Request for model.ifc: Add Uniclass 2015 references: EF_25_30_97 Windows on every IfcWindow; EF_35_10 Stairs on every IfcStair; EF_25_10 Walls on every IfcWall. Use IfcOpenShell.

First a look at what the model holds.

```python
import ifcopenshell

model = ifcopenshell.open("model.ifc")
print(model.schema)
print("classifications:", [c.Name for c in model.by_type("IfcClassification")])
for ifc_class in ("IfcDoor", "IfcRoof", "IfcStair", "IfcWall", "IfcWindow"):
    print(ifc_class, len(model.by_type(ifc_class)))
```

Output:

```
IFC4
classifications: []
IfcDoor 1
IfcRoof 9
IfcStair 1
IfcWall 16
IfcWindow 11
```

```python
import ifcopenshell
import ifcopenshell.api.classification

model = ifcopenshell.open("model.ifc")

system = ifcopenshell.api.classification.add_classification(model, classification="Uniclass 2015")

codes = {
    "IfcWindow": ("EF_25_30_97", "Windows"),
    "IfcStair": ("EF_35_10", "Stairs"),
    "IfcWall": ("EF_25_10", "Walls"),
}
for ifc_class, (code, name) in codes.items():
    products = model.by_type(ifc_class)
    ifcopenshell.api.classification.add_reference(
        model, products=products, classification=system, identification=code, name=name
    )
    print(code, len(products))

model.write("model-out.ifc")
```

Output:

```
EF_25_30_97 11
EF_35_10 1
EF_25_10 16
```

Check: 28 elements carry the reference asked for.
